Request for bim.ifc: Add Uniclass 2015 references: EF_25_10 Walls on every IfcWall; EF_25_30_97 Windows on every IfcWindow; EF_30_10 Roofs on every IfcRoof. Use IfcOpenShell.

First a look at what the model holds.

```python
import ifcopenshell

model = ifcopenshell.open("bim.ifc")
print(model.schema)
print("classifications:", [c.Name for c in model.by_type("IfcClassification")])
for ifc_class in ("IfcDoor", "IfcRoof", "IfcStair", "IfcWall", "IfcWindow"):
    print(ifc_class, len(model.by_type(ifc_class)))
```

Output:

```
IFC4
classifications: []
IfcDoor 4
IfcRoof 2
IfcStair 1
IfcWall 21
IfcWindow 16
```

```python
import ifcopenshell
import ifcopenshell.api.classification

model = ifcopenshell.open("bim.ifc")

system = ifcopenshell.api.classification.add_classification(model, classification="Uniclass 2015")

codes = {
    "IfcWall": ("EF_25_10", "Walls"),
    "IfcWindow": ("EF_25_30_97", "Windows"),
    "IfcRoof": ("EF_30_10", "Roofs"),
}
for ifc_class, (code, name) in codes.items():
    products = model.by_type(ifc_class)
    ifcopenshell.api.classification.add_reference(
        model, products=products, classification=system, identification=code, name=name
    )
    print(code, len(products))

model.write("bim-out.ifc")
```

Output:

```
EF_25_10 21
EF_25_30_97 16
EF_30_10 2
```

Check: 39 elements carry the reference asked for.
